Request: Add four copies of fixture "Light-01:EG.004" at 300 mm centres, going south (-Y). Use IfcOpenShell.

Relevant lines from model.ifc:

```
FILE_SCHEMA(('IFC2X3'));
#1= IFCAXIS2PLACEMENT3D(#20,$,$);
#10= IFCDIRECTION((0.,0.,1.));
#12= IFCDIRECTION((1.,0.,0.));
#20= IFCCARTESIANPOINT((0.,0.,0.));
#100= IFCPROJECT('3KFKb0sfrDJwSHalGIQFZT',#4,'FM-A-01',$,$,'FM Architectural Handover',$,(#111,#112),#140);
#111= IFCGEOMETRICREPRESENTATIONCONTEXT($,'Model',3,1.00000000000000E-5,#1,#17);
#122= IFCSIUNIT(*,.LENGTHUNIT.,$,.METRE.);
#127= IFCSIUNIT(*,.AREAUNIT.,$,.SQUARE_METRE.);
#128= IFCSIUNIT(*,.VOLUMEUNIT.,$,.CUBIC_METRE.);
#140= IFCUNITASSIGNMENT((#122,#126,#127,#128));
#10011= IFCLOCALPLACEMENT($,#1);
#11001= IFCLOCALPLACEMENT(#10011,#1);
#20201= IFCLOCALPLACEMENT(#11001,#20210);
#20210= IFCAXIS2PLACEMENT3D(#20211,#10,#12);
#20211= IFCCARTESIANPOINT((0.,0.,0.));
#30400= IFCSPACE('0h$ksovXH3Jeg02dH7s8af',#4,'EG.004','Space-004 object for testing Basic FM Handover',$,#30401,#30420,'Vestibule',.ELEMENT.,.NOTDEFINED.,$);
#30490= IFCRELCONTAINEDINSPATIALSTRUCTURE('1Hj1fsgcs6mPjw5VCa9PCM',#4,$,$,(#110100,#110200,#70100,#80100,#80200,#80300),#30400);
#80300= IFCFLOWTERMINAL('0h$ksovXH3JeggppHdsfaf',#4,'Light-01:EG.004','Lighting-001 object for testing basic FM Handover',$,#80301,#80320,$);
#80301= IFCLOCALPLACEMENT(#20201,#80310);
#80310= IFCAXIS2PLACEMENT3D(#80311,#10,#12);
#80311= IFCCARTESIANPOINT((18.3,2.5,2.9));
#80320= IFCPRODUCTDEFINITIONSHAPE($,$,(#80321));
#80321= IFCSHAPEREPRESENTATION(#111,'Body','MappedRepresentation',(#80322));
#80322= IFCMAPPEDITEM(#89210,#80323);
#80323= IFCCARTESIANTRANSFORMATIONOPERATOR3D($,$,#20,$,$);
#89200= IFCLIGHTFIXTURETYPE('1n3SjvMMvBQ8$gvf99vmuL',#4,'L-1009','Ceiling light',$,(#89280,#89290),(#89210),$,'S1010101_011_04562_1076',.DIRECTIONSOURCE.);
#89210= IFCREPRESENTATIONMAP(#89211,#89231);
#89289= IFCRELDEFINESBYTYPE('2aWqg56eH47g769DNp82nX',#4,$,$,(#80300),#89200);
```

```python
import numpy as np
import ifcopenshell
import ifcopenshell.api.geometry
import ifcopenshell.api.root
import ifcopenshell.util.element
import ifcopenshell.util.placement

model = ifcopenshell.open("model.ifc")

source = model.by_guid("0h$ksovXH3JeggppHdsfaf")
base = ifcopenshell.util.placement.get_local_placement(source.ObjectPlacement)
step = np.array([0.0, -1.0, 0.0]) * 0.3

for i in range(1, 5):
    copy = ifcopenshell.api.root.copy_class(model, product=source)
    copy.Representation = ifcopenshell.util.element.copy_deep(
        model, source.Representation, exclude=["IfcGeometricRepresentationContext", "IfcRepresentationMap"]
    )
    matrix = base.copy()
    matrix[:3, 3] += i * step
    print("added at", matrix[:3, 3].round(3) + 0.0)
    ifcopenshell.api.geometry.edit_object_placement(model, product=copy, matrix=matrix, is_si=False)

model.write("model-out.ifc")
```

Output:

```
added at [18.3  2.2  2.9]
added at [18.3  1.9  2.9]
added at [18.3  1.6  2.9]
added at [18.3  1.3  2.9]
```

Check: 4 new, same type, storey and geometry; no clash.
